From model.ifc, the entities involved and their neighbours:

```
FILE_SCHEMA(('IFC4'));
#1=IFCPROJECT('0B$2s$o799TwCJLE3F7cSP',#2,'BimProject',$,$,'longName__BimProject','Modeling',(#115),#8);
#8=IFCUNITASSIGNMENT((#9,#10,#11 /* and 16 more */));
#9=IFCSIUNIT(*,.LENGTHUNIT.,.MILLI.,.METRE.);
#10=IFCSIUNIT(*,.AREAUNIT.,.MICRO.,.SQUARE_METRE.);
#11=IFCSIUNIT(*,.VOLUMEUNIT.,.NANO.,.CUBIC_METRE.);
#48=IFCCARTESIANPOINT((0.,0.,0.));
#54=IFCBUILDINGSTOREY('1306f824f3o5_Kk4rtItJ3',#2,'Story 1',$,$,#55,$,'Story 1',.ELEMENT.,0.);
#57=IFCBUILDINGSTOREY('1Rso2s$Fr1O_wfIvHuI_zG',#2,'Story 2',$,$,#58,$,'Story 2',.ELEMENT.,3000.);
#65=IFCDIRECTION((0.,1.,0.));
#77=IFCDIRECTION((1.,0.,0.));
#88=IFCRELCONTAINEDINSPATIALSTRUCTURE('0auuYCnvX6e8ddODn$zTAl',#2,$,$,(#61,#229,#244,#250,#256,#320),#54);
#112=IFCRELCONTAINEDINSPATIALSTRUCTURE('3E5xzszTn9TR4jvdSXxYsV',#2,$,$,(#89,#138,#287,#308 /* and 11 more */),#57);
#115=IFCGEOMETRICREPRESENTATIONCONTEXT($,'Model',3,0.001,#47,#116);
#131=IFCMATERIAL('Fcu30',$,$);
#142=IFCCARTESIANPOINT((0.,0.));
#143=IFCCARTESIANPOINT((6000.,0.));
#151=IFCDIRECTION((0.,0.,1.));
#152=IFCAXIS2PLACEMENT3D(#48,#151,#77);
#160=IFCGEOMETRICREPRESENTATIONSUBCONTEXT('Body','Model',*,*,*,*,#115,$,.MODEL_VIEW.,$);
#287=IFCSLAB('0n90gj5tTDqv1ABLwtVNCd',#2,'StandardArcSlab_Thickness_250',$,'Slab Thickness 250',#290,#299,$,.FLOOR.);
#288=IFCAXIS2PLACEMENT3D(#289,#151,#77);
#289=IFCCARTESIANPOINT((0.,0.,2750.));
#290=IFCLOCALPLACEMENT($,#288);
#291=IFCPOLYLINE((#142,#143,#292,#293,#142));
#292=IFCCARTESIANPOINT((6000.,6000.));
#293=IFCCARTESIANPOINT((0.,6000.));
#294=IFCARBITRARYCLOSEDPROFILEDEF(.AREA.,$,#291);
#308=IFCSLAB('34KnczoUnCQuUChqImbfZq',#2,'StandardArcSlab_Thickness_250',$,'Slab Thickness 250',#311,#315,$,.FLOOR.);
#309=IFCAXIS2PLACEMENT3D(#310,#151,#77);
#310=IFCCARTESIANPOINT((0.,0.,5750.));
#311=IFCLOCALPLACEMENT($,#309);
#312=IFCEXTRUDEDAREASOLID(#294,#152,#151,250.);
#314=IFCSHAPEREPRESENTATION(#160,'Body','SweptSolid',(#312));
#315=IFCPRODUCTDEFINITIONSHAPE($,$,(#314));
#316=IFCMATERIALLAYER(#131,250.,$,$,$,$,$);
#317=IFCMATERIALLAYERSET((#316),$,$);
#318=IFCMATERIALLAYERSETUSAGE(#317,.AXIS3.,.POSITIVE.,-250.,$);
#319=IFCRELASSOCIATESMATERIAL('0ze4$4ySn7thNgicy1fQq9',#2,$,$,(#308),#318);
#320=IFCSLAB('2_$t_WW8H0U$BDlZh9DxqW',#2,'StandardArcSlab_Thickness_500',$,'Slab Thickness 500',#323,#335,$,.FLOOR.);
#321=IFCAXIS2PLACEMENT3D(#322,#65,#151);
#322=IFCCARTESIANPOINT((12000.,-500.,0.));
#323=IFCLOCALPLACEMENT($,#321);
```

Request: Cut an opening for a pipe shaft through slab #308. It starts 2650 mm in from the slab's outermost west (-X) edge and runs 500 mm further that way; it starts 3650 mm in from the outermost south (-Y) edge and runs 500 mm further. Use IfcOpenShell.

```python
import numpy as np
import ifcopenshell
import ifcopenshell.api.feature
import ifcopenshell.api.geometry
import ifcopenshell.api.root
import ifcopenshell.geom
import ifcopenshell.util.placement
import ifcopenshell.util.representation
import ifcopenshell.util.shape
import ifcopenshell.util.unit

model = ifcopenshell.open("model.ifc")
unit_scale = ifcopenshell.util.unit.calculate_unit_scale(model)
settings = ifcopenshell.geom.settings()


def volume(element):
    """Net volume in cubic metres, openings subtracted."""
    shape = ifcopenshell.geom.create_shape(settings, element)
    return ifcopenshell.util.shape.get_volume(shape.geometry)


slab = model.by_guid("34KnczoUnCQuUChqImbfZq")
before = volume(slab)

# Extent in the slab's own axes, in metres. The edges named are its -X and -Y sides.
slab_shape = ifcopenshell.geom.create_shape(settings, slab)
vertices = ifcopenshell.util.shape.get_vertices(slab_shape.geometry)
x_min, y_min, bottom = vertices.min(axis=0)
top = vertices[:, 2].max()

opening = ifcopenshell.api.root.create_entity(model, ifc_class="IfcOpeningElement", name="Pipe shaft opening", predefined_type="OPENING")
context = ifcopenshell.util.representation.get_context(model, "Model", "Body", "MODEL_VIEW")
width, depth = 0.5, 0.5
outline = [(0.0, 0.0), (width, 0.0), (width, depth), (0.0, depth), (0.0, 0.0)]
# Overshoot both faces by 50 mm so the cut is clean.
shape = ifcopenshell.api.geometry.add_slab_representation(
    model, context=context, depth=top - bottom + 0.1, polyline=outline
)
ifcopenshell.api.geometry.assign_representation(model, product=opening, representation=shape)

matrix = ifcopenshell.util.placement.get_local_placement(slab.ObjectPlacement)
matrix[:, 3] = matrix @ np.append(np.array([x_min + 2.65, y_min + 3.65, bottom - 0.05]) / unit_scale, 1.0)
ifcopenshell.api.geometry.edit_object_placement(model, product=opening, matrix=matrix, is_si=False)
ifcopenshell.api.feature.add_feature(model, feature=opening, element=slab)

after = volume(slab)

print(f"slab volume {before:.3f} -> {after:.3f} m3")

model.write("model_v2.ifc")
```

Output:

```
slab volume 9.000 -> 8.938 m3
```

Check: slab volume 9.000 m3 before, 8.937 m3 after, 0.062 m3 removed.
